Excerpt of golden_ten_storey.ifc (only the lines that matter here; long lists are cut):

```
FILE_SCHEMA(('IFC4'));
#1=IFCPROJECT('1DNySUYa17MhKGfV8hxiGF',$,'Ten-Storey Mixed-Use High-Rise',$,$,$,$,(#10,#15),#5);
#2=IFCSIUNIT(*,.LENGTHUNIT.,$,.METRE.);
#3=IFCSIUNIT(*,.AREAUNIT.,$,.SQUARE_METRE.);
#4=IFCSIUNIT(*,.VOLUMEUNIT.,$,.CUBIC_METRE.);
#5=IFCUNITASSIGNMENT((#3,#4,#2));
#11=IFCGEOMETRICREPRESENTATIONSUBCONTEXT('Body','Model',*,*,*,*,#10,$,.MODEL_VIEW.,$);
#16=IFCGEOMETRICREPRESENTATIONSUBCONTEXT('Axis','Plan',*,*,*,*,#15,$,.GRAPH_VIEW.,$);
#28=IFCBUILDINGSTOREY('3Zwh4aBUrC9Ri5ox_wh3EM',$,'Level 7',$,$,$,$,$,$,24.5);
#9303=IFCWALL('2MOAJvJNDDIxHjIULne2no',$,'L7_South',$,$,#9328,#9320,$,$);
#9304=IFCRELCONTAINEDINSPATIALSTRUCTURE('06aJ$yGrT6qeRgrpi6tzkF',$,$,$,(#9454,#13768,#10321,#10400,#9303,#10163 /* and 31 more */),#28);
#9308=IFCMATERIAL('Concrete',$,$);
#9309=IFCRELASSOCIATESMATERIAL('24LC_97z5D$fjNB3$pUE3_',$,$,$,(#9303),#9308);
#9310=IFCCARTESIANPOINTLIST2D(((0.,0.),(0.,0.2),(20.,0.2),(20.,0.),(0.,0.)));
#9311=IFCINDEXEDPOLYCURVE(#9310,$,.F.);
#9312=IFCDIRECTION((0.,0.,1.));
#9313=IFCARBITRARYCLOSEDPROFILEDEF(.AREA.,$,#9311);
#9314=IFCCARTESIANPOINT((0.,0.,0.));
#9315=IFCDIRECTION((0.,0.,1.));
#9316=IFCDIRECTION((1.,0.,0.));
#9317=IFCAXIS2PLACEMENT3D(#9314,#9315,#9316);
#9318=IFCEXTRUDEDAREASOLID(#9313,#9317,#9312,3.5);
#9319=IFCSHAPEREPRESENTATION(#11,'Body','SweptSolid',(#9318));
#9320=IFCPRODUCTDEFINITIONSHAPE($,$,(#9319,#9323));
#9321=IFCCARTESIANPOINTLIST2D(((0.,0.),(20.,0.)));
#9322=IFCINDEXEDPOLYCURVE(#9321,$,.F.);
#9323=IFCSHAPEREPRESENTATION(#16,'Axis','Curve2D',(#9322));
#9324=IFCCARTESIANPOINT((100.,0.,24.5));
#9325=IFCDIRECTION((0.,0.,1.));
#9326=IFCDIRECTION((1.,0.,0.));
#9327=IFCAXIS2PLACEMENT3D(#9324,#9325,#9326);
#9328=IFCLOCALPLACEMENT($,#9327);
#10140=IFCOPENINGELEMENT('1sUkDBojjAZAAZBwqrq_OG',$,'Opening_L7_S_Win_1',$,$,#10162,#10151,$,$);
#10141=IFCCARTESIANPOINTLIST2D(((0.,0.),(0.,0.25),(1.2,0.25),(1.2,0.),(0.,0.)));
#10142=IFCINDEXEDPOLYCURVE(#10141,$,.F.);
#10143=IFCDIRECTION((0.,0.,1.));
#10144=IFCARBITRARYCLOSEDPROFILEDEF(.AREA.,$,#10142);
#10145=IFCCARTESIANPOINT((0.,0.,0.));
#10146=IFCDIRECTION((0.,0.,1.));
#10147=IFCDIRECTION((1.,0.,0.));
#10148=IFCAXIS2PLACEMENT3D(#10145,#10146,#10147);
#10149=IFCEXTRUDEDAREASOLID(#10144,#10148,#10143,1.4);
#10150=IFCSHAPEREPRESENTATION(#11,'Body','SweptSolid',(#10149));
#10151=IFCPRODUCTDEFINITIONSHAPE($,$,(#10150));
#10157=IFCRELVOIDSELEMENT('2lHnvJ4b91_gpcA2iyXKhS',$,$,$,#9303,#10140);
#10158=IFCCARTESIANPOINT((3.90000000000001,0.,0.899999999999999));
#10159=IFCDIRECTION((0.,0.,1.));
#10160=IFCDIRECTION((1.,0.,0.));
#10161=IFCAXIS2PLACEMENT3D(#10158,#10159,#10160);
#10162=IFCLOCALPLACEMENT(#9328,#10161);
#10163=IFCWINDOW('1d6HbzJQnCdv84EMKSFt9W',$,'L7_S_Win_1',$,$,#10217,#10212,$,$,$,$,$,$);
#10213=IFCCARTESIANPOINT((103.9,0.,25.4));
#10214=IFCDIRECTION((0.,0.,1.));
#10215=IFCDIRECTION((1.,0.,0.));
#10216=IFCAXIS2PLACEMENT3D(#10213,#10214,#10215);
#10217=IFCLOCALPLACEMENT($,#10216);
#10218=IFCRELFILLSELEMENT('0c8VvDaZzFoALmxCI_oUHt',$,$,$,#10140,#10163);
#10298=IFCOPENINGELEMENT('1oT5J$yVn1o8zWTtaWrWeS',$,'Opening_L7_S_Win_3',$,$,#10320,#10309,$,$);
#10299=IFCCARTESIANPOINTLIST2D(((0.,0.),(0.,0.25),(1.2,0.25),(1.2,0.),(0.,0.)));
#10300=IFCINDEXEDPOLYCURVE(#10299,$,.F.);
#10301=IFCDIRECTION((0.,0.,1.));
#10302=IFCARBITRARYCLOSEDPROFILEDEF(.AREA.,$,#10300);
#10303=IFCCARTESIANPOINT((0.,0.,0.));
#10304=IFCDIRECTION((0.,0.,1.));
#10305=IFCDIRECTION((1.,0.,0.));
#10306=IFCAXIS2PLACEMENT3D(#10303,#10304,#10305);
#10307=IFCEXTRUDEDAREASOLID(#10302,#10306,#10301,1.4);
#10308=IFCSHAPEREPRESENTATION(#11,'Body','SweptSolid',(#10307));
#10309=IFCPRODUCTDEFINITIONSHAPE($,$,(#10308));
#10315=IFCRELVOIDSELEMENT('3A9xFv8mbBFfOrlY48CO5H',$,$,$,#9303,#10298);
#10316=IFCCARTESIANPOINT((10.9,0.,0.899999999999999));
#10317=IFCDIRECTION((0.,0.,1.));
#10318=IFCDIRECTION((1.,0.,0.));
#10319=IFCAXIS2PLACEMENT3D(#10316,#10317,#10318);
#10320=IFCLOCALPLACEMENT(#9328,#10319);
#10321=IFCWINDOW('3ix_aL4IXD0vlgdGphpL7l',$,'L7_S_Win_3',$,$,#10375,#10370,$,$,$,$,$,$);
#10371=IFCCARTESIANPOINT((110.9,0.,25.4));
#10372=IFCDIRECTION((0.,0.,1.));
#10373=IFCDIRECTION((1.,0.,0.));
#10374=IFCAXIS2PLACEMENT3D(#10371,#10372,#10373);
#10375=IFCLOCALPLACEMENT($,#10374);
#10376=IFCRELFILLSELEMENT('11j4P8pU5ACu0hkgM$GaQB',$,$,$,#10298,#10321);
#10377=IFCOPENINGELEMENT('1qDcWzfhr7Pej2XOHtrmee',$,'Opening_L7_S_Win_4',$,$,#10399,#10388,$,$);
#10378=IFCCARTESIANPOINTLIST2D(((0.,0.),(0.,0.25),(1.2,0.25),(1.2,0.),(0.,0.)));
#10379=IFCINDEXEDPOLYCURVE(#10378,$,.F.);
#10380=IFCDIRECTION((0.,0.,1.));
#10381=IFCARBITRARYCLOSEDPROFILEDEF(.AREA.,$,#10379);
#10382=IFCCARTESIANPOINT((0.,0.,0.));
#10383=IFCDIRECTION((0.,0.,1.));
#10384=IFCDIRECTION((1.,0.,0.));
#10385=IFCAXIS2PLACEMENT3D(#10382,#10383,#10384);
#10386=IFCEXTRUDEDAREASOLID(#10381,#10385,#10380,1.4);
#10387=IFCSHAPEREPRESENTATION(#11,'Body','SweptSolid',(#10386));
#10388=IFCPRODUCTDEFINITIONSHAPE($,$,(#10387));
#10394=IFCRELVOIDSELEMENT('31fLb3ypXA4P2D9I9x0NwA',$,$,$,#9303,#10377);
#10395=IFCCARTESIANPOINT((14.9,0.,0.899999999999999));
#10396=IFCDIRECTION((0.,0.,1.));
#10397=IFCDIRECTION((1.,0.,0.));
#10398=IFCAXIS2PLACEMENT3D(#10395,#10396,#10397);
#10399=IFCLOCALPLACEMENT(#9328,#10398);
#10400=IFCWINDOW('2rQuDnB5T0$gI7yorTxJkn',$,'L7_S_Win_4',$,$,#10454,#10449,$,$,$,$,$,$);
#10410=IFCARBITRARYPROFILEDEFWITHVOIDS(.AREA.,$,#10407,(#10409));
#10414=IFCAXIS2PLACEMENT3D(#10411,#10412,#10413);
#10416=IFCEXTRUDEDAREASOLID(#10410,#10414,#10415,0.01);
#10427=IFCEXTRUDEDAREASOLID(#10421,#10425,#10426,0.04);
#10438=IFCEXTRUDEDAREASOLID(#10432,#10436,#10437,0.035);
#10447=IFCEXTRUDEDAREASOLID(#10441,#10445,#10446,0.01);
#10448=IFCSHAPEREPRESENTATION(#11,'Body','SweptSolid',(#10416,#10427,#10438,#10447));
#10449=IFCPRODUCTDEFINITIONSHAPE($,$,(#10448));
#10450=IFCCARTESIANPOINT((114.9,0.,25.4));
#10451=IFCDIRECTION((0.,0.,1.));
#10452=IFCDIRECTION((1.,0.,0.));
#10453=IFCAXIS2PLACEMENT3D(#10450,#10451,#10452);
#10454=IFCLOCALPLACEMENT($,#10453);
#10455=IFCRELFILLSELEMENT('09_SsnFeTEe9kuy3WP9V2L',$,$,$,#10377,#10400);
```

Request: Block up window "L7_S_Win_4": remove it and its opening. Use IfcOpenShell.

```python
import ifcopenshell
import ifcopenshell.api.feature
import ifcopenshell.api.root
import ifcopenshell.geom
import ifcopenshell.util.shape

model = ifcopenshell.open("golden_ten_storey.ifc")
settings = ifcopenshell.geom.settings()


def volume(element):
    """Net volume in cubic metres, openings subtracted."""
    shape = ifcopenshell.geom.create_shape(settings, element)
    return ifcopenshell.util.shape.get_volume(shape.geometry)


window = model.by_id(10400)
opening = window.FillsVoids[0].RelatingOpeningElement
wall = opening.VoidsElements[0].RelatingBuildingElement
before = volume(wall)

ifcopenshell.api.root.remove_product(model, product=window)
ifcopenshell.api.feature.remove_feature(model, feature=opening)

after = volume(wall)

print(f"wall volume {before:.3f} -> {after:.3f} m3")

model.write("golden_ten_storey_v2.ifc")
```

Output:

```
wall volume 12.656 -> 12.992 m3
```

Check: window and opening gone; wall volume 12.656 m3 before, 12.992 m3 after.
